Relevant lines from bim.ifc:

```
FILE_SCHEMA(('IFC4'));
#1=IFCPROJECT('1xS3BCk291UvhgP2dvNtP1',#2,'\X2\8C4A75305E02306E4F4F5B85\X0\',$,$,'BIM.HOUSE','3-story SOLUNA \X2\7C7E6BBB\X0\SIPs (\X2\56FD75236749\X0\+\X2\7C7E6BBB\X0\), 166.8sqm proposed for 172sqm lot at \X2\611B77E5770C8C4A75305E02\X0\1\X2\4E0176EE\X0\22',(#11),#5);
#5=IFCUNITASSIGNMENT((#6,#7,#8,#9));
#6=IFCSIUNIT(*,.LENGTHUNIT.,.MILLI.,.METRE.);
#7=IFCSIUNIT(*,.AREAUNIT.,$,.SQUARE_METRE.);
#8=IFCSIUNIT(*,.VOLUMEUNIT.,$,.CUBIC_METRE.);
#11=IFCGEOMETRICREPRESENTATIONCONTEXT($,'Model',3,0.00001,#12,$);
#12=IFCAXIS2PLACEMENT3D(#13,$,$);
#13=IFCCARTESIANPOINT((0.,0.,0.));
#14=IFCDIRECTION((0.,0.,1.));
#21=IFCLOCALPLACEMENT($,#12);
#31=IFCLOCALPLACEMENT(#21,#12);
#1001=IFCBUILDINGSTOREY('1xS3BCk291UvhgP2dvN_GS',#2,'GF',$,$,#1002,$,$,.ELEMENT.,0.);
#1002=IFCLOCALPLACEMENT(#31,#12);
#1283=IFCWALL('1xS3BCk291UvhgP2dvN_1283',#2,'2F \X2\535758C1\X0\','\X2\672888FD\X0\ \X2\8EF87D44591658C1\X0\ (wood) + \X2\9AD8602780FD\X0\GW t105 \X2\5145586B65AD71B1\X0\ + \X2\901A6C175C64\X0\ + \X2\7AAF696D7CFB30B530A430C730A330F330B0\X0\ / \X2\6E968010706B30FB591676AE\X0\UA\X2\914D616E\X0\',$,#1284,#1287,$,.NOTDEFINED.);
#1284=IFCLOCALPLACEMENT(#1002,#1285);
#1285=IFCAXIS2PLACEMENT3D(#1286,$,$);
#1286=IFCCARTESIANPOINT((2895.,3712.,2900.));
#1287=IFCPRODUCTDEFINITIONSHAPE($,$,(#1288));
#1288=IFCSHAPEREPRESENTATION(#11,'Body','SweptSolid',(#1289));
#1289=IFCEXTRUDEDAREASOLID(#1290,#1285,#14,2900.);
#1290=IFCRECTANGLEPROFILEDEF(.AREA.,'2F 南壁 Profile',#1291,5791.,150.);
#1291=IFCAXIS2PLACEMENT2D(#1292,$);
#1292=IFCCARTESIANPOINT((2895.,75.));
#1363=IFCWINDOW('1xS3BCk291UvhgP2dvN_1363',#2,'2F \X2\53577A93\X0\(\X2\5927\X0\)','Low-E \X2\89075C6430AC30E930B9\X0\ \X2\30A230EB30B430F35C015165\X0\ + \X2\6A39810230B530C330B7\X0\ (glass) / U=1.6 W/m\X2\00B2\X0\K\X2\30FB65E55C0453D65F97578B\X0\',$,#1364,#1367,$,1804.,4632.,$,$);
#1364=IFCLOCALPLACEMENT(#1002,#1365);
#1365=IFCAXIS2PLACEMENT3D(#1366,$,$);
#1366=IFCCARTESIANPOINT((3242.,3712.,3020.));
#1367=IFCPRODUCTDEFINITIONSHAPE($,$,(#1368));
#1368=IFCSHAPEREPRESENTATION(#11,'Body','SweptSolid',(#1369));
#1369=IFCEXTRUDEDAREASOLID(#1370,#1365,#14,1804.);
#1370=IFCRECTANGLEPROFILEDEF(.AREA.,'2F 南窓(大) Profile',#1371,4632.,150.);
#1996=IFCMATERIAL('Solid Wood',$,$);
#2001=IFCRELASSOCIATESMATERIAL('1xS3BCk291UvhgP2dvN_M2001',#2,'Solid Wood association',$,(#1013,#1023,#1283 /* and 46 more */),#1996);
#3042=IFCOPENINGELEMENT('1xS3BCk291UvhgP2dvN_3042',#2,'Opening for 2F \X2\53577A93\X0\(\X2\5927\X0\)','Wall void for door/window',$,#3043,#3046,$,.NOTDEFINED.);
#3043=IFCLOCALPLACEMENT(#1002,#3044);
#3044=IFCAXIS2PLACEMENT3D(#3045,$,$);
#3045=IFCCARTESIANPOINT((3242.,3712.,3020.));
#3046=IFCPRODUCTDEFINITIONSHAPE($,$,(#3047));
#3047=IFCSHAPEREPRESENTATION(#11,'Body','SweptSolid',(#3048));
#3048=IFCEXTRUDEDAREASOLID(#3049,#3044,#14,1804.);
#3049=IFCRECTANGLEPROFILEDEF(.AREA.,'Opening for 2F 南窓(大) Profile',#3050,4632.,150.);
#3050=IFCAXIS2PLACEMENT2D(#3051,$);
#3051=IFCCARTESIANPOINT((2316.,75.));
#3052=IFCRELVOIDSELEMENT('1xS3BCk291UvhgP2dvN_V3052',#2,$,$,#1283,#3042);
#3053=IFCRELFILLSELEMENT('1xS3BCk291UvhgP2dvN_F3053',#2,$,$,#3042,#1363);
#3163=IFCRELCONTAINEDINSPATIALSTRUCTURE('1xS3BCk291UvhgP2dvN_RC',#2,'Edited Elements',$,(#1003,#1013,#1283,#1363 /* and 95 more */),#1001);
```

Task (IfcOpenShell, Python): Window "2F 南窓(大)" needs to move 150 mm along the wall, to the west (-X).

```python
import ifcopenshell
import ifcopenshell.api.geometry
import ifcopenshell.util.placement
import ifcopenshell.util.unit

model = ifcopenshell.open("bim.ifc")
unit_scale = ifcopenshell.util.unit.calculate_unit_scale(model)

window = model.by_guid("1xS3BCk291UvhgP2dvN_1363")
opening = window.FillsVoids[0].RelatingOpeningElement
wall = opening.VoidsElements[0].RelatingBuildingElement

wall_matrix = ifcopenshell.util.placement.get_local_placement(wall.ObjectPlacement)
shift = wall_matrix[:3, 0] * -0.15 / unit_scale
before = ifcopenshell.util.placement.get_local_placement(window.ObjectPlacement)[:3, 3].copy()

# The window is not placed relative to its opening, so move both.
for product in (opening, window):
    matrix = ifcopenshell.util.placement.get_local_placement(product.ObjectPlacement)
    matrix[:3, 3] += shift
    ifcopenshell.api.geometry.edit_object_placement(model, product=product, matrix=matrix, is_si=False)

after = ifcopenshell.util.placement.get_local_placement(window.ObjectPlacement)[:3, 3]
print("window moved by", (after - before).round(3) + 0.0)

model.write("bim-out.ifc")
```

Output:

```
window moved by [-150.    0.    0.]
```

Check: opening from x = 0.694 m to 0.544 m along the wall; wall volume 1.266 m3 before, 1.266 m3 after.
